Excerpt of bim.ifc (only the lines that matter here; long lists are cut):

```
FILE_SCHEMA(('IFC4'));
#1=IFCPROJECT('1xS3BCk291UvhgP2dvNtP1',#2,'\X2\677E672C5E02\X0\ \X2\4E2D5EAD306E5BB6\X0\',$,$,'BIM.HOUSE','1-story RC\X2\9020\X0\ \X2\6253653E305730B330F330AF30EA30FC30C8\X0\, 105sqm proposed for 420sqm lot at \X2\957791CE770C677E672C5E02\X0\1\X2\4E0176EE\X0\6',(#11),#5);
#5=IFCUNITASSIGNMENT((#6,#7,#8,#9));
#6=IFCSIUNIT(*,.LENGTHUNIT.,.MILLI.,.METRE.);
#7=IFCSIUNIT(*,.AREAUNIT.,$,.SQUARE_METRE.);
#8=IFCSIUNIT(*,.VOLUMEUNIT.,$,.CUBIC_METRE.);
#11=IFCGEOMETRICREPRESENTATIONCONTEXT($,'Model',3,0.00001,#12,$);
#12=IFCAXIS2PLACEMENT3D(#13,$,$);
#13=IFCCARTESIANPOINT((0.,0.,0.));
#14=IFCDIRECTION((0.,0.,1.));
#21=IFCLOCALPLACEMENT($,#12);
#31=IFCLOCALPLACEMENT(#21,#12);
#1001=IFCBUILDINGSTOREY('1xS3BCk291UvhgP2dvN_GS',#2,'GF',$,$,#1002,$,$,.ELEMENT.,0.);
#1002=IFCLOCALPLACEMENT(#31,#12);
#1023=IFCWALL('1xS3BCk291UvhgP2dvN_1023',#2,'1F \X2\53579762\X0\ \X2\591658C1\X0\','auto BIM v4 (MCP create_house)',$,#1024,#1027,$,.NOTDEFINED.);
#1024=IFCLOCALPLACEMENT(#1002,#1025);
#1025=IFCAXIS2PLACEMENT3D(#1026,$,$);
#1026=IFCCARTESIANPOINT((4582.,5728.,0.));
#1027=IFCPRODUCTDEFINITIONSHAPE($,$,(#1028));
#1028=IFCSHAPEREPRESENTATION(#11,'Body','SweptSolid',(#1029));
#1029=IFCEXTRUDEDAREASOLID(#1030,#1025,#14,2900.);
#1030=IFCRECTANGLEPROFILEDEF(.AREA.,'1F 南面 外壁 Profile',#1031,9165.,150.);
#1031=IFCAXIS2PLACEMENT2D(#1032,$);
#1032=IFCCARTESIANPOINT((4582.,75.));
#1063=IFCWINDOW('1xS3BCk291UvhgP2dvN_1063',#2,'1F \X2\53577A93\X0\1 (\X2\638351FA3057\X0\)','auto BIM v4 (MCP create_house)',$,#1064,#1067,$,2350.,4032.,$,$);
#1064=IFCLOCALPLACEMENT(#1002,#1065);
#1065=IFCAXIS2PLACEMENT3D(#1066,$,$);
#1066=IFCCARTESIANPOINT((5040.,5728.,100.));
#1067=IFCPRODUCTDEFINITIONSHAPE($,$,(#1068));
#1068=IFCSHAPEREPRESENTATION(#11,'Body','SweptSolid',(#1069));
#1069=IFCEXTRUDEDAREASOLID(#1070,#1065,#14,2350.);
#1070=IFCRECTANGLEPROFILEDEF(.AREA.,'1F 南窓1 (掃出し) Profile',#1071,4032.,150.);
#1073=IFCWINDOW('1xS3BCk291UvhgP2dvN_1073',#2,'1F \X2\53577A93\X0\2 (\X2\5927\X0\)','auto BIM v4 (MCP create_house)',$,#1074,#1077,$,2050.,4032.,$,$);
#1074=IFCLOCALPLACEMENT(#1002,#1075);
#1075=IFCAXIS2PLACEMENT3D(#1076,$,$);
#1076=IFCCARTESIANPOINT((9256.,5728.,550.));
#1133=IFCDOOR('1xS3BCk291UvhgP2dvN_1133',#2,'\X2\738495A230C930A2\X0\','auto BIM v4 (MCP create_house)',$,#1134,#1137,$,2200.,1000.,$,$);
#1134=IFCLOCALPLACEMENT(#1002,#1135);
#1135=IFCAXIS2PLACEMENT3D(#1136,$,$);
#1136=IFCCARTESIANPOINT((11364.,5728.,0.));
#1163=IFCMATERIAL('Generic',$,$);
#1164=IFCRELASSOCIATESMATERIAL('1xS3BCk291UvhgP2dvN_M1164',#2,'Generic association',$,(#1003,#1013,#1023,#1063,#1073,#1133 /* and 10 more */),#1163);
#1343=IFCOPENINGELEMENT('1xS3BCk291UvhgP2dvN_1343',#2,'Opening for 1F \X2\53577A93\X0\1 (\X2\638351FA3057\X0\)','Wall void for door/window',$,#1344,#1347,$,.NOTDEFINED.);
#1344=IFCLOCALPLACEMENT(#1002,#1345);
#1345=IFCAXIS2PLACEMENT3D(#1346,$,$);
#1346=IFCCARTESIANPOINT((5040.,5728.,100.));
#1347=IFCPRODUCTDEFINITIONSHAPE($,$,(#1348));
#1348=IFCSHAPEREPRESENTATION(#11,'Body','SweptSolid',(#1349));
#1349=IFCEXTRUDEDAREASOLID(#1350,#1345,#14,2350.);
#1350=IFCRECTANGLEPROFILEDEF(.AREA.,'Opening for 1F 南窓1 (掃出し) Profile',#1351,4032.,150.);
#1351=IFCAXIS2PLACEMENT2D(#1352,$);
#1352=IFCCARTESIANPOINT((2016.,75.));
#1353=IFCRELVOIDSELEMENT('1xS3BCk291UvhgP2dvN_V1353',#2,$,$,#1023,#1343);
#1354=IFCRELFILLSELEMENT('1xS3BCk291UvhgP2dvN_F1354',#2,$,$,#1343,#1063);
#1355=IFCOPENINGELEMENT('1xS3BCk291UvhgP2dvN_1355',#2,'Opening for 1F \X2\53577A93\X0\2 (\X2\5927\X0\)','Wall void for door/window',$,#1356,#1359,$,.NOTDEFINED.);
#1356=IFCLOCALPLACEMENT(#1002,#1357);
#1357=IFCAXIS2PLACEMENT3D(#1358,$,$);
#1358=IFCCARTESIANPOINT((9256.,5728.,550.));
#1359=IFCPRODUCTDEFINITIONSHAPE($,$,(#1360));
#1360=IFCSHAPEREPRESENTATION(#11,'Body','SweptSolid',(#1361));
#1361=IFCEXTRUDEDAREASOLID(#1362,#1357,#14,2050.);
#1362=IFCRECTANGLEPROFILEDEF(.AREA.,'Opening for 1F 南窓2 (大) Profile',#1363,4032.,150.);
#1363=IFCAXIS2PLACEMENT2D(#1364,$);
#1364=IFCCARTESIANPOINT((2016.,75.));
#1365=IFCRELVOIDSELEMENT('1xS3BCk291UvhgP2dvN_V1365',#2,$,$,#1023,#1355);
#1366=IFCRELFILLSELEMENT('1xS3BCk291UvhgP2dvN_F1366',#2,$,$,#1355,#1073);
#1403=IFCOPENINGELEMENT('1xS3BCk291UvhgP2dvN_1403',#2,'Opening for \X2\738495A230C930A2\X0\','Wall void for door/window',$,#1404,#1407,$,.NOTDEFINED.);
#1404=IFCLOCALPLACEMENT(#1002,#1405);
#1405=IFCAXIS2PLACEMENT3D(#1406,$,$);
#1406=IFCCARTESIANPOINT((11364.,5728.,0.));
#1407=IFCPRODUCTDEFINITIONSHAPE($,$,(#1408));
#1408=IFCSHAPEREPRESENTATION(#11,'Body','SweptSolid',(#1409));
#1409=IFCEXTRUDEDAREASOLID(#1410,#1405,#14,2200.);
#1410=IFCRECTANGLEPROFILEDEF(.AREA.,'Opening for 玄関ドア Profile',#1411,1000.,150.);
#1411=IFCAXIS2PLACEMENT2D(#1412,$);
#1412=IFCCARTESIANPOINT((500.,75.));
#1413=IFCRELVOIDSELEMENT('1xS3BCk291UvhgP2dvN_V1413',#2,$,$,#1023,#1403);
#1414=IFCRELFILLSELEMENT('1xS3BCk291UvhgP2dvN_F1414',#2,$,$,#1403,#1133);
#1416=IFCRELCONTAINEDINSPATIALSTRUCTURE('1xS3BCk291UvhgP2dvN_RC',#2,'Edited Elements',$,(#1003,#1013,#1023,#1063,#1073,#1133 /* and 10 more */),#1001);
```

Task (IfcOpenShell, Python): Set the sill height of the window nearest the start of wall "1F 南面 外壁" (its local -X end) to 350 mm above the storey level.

```python
import numpy as np
import ifcopenshell
import ifcopenshell.api.geometry
import ifcopenshell.geom
import ifcopenshell.util.element
import ifcopenshell.util.placement
import ifcopenshell.util.shape
import ifcopenshell.util.unit

model = ifcopenshell.open("bim.ifc")
unit_scale = ifcopenshell.util.unit.calculate_unit_scale(model)

window = model.by_guid("1xS3BCk291UvhgP2dvN_1063")
opening = window.FillsVoids[0].RelatingOpeningElement
storey = ifcopenshell.util.element.get_container(window, ifc_class="IfcBuildingStorey")
level = ifcopenshell.util.placement.get_local_placement(storey.ObjectPlacement)[2, 3]

# The opening's origin need not be at the sill, so measure its lowest point.
shape = ifcopenshell.geom.create_shape(ifcopenshell.geom.settings(), opening)
bottom = ifcopenshell.util.shape.get_shape_bottom_elevation(shape, shape.geometry) / unit_scale
dz = level + 0.35 / unit_scale - bottom

shift = np.array([0.0, 0.0, dz])
# The window is not placed relative to its opening, so move both.
for product in (opening, window):
    matrix = ifcopenshell.util.placement.get_local_placement(product.ObjectPlacement)
    matrix[:3, 3] += shift
    ifcopenshell.api.geometry.edit_object_placement(model, product=product, matrix=matrix, is_si=False)

print(f"moved by {dz * unit_scale:+.3f} m")

model.write("bim_edited.ifc")
```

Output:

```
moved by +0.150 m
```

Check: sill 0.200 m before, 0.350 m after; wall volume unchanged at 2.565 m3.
